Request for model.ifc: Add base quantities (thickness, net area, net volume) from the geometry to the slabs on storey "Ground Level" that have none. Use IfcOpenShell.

First a look at what the model holds.

```python
import ifcopenshell
import ifcopenshell.util.element
import ifcopenshell.util.unit

model = ifcopenshell.open("model.ifc")
print(model.schema)
for unit_type in ("LENGTHUNIT", "AREAUNIT", "VOLUMEUNIT"):
    print(unit_type, ifcopenshell.util.unit.calculate_unit_scale(model, unit_type))
storey = next(s for s in model.by_type("IfcBuildingStorey") if s.Name == "Ground Level")
slabs = [e for e in ifcopenshell.util.element.get_decomposition(storey) if e.is_a("IfcSlab")]
for e in sorted(slabs, key=lambda e: e.id()):
    print(e.id(), e.is_a(), e.Name, list(ifcopenshell.util.element.get_psets(e, qtos_only=True)), sep=" | ")
```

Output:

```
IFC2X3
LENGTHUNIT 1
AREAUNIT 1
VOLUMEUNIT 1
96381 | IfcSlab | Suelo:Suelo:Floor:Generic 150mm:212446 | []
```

```python
import ifcopenshell
import ifcopenshell.api.pset
import ifcopenshell.geom
import ifcopenshell.util.element
import ifcopenshell.util.shape
import ifcopenshell.util.unit

model = ifcopenshell.open("model.ifc")
unit_scale = ifcopenshell.util.unit.calculate_unit_scale(model)
area_scale = ifcopenshell.util.unit.calculate_unit_scale(model, "AREAUNIT")
volume_scale = ifcopenshell.util.unit.calculate_unit_scale(model, "VOLUMEUNIT")
settings = ifcopenshell.geom.settings()

storey = next(s for s in model.by_type("IfcBuildingStorey") if s.Name == "Ground Level")
slabs = [e for e in ifcopenshell.util.element.get_decomposition(storey) if e.is_a("IfcSlab")]

for e in sorted(slabs, key=lambda e: e.id()):
    if ifcopenshell.util.element.get_psets(e, qtos_only=True, should_inherit=False):
        continue
    # Geometry comes back in metres, in the element's own axes.
    shape = ifcopenshell.geom.create_shape(settings, e)
    values = {
        "Width": ifcopenshell.util.shape.get_z(shape.geometry) / unit_scale,
        "NetArea": ifcopenshell.util.shape.get_footprint_area(shape.geometry) / area_scale,
        "NetVolume": ifcopenshell.util.shape.get_volume(shape.geometry) / volume_scale,
    }
    qto = ifcopenshell.api.pset.add_qto(model, product=e, name="BaseQuantities")
    ifcopenshell.api.pset.edit_qto(model, qto=qto, properties=values)
    print(e.id(), {k: round(v, 3) for k, v in values.items()})

model.write("model_edited.ifc")
```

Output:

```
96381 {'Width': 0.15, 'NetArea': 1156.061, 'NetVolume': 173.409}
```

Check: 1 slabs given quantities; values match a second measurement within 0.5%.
